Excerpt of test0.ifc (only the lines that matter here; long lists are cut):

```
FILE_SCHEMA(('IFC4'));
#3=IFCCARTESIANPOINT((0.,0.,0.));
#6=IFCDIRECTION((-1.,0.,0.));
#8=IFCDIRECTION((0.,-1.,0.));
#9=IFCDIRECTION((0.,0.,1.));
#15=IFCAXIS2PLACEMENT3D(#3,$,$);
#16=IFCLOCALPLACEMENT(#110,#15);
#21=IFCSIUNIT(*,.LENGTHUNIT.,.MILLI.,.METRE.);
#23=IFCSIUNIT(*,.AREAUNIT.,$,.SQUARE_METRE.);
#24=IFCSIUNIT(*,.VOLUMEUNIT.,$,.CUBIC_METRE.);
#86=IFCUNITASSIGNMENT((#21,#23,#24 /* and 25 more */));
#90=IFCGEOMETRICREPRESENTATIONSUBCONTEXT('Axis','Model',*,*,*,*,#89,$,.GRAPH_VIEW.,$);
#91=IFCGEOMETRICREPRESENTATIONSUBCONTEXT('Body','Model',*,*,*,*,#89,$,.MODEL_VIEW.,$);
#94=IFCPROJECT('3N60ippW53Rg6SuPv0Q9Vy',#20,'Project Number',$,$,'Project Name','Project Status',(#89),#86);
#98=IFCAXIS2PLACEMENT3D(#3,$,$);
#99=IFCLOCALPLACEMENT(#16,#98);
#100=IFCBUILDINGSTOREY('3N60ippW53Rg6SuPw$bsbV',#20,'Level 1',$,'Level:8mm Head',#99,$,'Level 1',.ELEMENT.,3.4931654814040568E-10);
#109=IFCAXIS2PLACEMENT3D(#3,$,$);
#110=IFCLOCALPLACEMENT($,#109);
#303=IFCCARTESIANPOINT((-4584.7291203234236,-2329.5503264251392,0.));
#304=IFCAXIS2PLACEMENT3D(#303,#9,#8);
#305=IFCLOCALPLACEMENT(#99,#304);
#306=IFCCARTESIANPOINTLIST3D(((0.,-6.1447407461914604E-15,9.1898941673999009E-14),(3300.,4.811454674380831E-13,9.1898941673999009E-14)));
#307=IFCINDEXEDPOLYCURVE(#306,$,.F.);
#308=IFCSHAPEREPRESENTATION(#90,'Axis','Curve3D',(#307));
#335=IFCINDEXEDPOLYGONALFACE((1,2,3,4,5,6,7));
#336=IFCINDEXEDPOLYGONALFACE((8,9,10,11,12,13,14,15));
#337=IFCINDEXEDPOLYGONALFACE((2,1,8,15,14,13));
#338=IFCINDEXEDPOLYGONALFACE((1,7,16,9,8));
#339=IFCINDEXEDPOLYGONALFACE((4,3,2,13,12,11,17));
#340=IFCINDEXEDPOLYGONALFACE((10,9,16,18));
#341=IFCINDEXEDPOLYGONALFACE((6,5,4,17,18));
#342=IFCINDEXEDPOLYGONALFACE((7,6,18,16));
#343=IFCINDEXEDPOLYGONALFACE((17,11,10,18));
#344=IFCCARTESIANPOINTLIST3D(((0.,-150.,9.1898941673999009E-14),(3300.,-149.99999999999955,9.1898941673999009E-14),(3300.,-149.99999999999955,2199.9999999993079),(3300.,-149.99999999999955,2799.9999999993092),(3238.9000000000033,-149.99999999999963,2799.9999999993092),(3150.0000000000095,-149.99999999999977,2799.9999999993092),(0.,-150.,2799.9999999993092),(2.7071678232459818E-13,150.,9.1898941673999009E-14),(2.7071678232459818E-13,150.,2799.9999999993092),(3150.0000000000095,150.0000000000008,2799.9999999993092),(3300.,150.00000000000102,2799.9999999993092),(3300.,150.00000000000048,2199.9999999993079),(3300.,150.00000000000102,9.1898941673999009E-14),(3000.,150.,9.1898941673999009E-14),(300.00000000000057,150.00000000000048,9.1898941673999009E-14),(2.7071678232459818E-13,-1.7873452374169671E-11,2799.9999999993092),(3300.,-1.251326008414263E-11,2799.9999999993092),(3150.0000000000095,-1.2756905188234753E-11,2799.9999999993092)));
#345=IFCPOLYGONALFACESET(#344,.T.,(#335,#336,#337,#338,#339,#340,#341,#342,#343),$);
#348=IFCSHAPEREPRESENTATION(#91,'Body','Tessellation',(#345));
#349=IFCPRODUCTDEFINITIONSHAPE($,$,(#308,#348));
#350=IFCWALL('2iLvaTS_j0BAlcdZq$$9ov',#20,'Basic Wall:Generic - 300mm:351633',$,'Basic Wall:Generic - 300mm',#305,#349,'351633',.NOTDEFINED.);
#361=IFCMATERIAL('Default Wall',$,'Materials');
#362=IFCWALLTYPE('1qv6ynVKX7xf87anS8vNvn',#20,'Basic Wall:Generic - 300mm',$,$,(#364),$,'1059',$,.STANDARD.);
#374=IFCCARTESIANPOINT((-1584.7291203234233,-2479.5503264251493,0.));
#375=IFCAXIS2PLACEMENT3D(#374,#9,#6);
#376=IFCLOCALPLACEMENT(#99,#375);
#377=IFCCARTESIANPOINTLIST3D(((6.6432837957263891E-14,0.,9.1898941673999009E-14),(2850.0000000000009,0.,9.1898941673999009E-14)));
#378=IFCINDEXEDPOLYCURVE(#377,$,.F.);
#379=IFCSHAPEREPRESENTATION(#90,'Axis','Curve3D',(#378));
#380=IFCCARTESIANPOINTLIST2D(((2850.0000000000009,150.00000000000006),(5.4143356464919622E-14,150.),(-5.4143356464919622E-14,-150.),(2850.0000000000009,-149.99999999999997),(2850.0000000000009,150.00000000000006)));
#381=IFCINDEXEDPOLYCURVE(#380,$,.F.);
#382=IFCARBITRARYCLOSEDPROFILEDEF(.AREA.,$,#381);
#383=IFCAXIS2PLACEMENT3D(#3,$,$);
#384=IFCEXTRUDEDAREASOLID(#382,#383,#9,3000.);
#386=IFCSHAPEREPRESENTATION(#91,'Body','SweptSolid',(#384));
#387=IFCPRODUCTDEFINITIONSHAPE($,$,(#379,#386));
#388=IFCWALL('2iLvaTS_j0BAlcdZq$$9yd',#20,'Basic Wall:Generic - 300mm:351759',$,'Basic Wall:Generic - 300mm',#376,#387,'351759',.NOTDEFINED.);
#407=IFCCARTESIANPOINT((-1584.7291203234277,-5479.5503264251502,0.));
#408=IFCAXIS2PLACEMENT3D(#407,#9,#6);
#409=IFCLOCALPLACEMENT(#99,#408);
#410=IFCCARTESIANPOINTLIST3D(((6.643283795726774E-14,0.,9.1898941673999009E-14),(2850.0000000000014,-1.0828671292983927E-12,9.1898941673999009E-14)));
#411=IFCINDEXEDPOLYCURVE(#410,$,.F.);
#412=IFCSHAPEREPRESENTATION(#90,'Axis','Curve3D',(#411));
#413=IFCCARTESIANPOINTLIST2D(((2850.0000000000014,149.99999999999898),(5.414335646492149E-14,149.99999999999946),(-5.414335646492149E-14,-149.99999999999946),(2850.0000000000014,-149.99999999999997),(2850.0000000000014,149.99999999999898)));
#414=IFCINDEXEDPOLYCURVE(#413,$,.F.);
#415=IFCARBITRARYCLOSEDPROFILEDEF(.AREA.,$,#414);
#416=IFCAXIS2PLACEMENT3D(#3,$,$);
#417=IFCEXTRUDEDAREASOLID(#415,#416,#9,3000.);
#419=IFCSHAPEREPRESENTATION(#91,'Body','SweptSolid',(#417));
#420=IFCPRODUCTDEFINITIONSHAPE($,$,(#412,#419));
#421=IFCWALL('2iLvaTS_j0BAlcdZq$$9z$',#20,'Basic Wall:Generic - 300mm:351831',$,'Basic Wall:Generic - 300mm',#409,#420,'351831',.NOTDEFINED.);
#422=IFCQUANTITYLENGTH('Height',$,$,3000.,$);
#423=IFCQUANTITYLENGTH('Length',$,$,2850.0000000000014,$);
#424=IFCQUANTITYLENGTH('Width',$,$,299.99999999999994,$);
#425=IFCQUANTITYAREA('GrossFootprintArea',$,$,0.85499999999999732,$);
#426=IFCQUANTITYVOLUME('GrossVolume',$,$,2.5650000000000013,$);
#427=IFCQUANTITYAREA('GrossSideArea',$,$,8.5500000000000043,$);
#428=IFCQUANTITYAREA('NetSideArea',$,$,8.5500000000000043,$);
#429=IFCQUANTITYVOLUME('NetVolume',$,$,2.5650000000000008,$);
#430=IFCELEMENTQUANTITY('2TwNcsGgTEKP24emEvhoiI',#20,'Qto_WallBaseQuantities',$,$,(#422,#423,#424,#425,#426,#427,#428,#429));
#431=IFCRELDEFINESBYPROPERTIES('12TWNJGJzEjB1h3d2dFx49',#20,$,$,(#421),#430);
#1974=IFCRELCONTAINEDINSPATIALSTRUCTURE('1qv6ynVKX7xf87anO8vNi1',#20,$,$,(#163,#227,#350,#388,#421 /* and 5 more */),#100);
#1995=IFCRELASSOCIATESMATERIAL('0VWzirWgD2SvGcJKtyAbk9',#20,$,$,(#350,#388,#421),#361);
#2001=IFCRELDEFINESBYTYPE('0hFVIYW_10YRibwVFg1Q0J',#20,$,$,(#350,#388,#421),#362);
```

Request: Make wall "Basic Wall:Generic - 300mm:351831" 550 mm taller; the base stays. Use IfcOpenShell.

```python
import ifcopenshell
import ifcopenshell.api.pset
import ifcopenshell.geom
import ifcopenshell.util.element
import ifcopenshell.util.representation
import ifcopenshell.util.shape
import ifcopenshell.util.unit

model = ifcopenshell.open("test0.ifc")
unit_scale = ifcopenshell.util.unit.calculate_unit_scale(model)
area_scale = ifcopenshell.util.unit.calculate_unit_scale(model, "AREAUNIT")
volume_scale = ifcopenshell.util.unit.calculate_unit_scale(model, "VOLUMEUNIT")
settings = ifcopenshell.geom.settings()


def volume(element):
    """Net volume in cubic metres, openings subtracted."""
    shape = ifcopenshell.geom.create_shape(settings, element)
    return ifcopenshell.util.shape.get_volume(shape.geometry)


wall = model.by_guid("2iLvaTS_j0BAlcdZq$$9z$")
before = volume(wall)

body = ifcopenshell.util.representation.get_representation(wall, "Model", "Body")
solid = body.Items[0]
old_height = solid.Depth
solid.Depth += 0.55 / unit_scale
after = volume(wall)
thickness = 0.3  # wall thickness in metres

# Update the stored height, areas and volumes.
qto = model.by_id(ifcopenshell.util.element.get_pset(wall, "Qto_WallBaseQuantities", should_inherit=False)["id"])
ifcopenshell.api.pset.edit_qto(model, qto=qto, properties={
    "Height": solid.Depth,
    "GrossVolume": ifcopenshell.util.element.get_pset(wall, "Qto_WallBaseQuantities", "GrossVolume") * solid.Depth / old_height,
    "GrossSideArea": ifcopenshell.util.element.get_pset(wall, "Qto_WallBaseQuantities", "GrossSideArea") * solid.Depth / old_height,
    "NetSideArea": after / thickness / area_scale,
    "NetVolume": after / volume_scale,
})

print(f"height {old_height:g} -> {solid.Depth:g}, volume {before:.3f} -> {after:.3f} m3")

model.write("test0_v2.ifc")
```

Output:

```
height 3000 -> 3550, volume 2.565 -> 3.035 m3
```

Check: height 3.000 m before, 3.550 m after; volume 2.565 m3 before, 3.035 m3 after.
